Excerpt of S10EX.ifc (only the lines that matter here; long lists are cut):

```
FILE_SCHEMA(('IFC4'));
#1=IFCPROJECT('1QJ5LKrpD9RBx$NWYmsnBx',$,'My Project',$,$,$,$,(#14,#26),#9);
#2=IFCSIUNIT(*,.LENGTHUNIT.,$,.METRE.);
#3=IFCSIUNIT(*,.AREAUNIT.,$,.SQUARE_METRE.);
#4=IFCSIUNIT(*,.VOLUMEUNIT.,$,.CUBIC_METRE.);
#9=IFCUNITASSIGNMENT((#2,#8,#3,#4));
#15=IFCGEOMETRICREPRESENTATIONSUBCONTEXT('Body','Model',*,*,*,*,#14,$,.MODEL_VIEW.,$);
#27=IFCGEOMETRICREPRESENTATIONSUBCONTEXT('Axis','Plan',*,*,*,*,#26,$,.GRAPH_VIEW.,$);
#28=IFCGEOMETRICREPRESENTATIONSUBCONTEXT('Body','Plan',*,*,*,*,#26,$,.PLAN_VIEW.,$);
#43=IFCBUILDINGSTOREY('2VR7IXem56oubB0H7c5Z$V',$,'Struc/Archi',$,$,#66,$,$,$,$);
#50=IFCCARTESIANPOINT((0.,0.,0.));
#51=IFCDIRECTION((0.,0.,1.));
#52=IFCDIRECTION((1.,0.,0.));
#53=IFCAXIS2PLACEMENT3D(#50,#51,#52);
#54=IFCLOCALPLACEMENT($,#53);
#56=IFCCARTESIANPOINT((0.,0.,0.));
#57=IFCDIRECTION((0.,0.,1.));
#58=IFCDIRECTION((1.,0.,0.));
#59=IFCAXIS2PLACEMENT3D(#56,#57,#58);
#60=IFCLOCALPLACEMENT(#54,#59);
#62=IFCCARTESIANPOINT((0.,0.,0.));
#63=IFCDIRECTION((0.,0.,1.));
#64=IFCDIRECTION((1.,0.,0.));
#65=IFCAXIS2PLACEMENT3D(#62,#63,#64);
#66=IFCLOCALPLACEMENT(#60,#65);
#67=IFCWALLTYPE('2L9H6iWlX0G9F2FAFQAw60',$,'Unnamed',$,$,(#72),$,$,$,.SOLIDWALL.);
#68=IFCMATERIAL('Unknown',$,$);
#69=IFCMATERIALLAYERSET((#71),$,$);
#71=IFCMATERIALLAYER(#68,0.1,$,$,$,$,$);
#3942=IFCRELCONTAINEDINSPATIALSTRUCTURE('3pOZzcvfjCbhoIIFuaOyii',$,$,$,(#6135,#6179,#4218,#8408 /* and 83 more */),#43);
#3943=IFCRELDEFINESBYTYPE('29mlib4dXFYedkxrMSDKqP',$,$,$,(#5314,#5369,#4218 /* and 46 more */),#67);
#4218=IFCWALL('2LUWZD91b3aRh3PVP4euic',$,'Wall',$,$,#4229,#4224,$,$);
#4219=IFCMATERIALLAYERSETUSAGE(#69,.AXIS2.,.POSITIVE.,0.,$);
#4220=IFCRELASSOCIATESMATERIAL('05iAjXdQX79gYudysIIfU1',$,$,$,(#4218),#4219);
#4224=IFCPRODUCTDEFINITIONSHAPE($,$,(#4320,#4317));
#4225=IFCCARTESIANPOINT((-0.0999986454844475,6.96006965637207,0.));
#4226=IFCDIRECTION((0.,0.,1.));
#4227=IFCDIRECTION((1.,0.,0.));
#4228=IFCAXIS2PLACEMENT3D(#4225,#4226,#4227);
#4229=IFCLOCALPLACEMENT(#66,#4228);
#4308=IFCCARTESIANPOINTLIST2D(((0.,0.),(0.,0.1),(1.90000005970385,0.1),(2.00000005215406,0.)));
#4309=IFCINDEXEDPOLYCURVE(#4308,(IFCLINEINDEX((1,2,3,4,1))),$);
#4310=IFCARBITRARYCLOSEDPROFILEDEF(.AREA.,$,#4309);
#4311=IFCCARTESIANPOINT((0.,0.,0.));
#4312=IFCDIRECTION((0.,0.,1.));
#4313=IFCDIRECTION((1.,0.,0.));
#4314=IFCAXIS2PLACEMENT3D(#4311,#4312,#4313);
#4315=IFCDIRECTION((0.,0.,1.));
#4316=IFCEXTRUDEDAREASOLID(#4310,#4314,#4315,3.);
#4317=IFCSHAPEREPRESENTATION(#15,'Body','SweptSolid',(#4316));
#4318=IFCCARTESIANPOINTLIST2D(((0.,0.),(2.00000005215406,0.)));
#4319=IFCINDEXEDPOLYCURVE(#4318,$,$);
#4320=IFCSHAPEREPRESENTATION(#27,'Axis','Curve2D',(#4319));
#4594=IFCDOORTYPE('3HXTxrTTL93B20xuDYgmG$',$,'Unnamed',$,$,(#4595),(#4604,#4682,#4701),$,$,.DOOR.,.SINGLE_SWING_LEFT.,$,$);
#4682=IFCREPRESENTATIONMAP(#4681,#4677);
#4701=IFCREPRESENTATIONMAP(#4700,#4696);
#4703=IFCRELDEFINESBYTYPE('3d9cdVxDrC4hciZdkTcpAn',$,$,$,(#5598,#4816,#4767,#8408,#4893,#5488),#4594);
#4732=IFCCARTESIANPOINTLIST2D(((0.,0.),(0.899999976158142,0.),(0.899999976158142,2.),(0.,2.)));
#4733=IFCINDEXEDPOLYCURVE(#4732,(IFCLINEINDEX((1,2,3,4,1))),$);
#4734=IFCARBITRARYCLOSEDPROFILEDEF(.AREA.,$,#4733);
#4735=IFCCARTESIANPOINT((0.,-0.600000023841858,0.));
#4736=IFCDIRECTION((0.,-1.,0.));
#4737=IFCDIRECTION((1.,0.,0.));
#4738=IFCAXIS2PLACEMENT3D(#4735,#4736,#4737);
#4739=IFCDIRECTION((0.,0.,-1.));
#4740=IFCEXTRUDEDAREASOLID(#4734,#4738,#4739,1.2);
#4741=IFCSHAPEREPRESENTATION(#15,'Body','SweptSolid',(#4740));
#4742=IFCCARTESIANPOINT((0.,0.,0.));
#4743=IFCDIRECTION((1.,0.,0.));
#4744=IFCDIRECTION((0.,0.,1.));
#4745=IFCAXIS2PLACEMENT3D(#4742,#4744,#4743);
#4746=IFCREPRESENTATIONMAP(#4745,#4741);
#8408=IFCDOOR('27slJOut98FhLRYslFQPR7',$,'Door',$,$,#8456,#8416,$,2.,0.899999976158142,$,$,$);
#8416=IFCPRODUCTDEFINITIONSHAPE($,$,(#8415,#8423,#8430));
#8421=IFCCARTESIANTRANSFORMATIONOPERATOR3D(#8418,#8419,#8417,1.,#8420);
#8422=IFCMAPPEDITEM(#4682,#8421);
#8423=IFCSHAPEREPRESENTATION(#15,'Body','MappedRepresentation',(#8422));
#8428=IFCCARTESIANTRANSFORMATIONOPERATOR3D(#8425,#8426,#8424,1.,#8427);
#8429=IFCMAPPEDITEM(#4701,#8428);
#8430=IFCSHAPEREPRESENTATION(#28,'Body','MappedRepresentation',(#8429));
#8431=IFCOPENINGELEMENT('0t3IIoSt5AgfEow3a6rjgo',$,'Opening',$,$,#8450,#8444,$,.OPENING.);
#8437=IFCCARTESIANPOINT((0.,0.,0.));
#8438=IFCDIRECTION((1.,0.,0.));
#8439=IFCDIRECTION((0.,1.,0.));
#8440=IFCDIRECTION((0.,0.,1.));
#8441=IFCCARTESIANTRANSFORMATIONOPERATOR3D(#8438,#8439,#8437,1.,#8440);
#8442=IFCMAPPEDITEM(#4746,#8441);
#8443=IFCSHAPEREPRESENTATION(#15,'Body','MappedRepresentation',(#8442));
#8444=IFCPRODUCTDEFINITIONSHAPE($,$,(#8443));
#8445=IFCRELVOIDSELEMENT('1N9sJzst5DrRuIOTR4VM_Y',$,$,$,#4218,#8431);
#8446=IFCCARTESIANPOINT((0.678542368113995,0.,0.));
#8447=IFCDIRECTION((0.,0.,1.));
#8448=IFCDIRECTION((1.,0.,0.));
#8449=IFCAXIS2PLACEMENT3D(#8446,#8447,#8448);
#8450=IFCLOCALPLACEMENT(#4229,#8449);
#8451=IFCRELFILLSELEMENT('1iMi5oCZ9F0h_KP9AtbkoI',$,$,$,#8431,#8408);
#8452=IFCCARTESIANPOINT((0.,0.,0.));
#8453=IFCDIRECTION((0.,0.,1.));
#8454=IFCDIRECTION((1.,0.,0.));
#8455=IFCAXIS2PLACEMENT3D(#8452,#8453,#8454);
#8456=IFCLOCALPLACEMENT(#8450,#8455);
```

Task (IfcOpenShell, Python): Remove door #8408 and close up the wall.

```python
import ifcopenshell
import ifcopenshell.api.feature
import ifcopenshell.api.root
import ifcopenshell.geom
import ifcopenshell.util.shape

model = ifcopenshell.open("S10EX.ifc")
settings = ifcopenshell.geom.settings()


def volume(element):
    """Net volume in cubic metres, openings subtracted."""
    shape = ifcopenshell.geom.create_shape(settings, element)
    return ifcopenshell.util.shape.get_volume(shape.geometry)


door = model.by_guid("27slJOut98FhLRYslFQPR7")
opening = door.FillsVoids[0].RelatingOpeningElement
wall = opening.VoidsElements[0].RelatingBuildingElement
before = volume(wall)

ifcopenshell.api.root.remove_product(model, product=door)
ifcopenshell.api.feature.remove_feature(model, feature=opening)

after = volume(wall)

print(f"wall volume {before:.3f} -> {after:.3f} m3")

model.write("S10EX_v2.ifc")
```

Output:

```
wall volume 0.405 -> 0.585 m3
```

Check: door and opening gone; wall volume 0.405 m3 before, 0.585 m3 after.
